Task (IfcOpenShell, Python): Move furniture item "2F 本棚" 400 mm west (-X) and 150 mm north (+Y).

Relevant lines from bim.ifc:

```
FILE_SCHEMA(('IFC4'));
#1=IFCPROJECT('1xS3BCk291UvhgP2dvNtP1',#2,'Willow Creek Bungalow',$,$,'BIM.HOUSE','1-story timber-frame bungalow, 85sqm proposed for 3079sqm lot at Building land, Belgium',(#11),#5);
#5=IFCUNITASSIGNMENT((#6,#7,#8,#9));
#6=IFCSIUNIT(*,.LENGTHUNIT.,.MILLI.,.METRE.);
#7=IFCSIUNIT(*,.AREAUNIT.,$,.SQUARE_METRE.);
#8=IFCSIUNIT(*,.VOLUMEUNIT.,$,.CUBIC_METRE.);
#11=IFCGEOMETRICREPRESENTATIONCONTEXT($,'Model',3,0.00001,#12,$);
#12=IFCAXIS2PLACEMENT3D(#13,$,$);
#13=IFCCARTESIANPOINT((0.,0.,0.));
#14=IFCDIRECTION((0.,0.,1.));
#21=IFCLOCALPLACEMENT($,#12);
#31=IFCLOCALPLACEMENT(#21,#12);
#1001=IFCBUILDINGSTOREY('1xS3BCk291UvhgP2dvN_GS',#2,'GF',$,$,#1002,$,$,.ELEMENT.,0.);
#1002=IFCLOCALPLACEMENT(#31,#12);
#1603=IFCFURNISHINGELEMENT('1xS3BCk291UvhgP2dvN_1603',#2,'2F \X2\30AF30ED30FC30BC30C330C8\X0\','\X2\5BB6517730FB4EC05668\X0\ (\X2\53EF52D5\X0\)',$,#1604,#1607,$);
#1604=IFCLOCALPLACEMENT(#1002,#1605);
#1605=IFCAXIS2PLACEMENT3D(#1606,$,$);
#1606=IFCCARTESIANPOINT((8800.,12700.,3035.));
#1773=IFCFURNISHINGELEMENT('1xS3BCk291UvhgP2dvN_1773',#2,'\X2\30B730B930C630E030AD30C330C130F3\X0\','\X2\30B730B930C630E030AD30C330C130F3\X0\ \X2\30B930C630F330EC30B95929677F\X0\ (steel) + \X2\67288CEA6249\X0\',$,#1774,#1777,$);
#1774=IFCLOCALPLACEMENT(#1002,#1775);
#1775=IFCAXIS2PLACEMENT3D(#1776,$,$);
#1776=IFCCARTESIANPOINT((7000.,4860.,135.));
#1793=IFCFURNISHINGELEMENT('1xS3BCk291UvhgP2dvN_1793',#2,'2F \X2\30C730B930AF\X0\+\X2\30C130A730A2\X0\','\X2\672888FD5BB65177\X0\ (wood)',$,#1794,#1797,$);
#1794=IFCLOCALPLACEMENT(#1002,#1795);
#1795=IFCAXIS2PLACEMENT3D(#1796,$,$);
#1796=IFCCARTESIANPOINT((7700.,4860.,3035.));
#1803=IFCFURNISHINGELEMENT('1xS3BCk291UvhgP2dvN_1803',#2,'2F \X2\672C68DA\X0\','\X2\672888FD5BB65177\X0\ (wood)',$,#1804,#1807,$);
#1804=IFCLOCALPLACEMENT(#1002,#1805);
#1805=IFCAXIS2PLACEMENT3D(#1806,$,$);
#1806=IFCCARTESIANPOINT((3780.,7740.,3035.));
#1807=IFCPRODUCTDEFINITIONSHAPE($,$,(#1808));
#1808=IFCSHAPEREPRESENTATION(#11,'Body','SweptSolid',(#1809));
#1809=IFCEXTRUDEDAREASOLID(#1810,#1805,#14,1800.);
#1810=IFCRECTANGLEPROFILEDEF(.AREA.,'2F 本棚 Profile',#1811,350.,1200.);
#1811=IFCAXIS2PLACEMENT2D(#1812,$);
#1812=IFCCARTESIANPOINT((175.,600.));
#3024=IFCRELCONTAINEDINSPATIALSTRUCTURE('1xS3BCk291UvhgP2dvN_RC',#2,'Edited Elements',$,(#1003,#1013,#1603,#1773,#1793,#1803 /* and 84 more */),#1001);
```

```python
import ifcopenshell
import ifcopenshell.api.geometry
import ifcopenshell.util.placement
import ifcopenshell.util.unit

model = ifcopenshell.open("bim.ifc")
unit_scale = ifcopenshell.util.unit.calculate_unit_scale(model)

item = model.by_guid("1xS3BCk291UvhgP2dvN_1803")
matrix = ifcopenshell.util.placement.get_local_placement(item.ObjectPlacement)
matrix[0, 3] -= 0.4 / unit_scale
matrix[1, 3] += 0.15 / unit_scale
ifcopenshell.api.geometry.edit_object_placement(model, product=item, matrix=matrix, is_si=False)

print(ifcopenshell.util.placement.get_local_placement(item.ObjectPlacement).round(3) + 0.0)

model.write("bim_updated.ifc")
```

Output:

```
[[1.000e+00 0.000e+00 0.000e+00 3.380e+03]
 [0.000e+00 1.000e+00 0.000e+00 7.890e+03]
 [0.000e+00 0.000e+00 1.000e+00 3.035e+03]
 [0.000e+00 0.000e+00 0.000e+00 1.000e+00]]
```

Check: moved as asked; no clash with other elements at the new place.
